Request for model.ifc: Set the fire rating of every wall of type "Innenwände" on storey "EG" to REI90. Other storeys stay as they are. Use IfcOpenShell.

First a look at what the model holds.

```python
import ifcopenshell
import ifcopenshell.util.element

model = ifcopenshell.open("model.ifc")
print(model.schema)
storey = next(s for s in model.by_type("IfcBuildingStorey") if s.Name == "EG")
walls = [e for e in ifcopenshell.util.element.get_decomposition(storey) if e.is_a("IfcWall")]
seen = {}
for e in walls:
    element_type = ifcopenshell.util.element.get_type(e)
    key = (element_type.Name if element_type != e and element_type else None, ifcopenshell.util.element.get_pset(e, "Pset_WallCommon", "FireRating"))
    seen[key] = seen.get(key, 0) + 1
for (name, value), count in sorted(seen.items(), key=str):
    print(count, "x", name, "|", value)
```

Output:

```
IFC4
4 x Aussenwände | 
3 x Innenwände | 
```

```python
import ifcopenshell
import ifcopenshell.api.pset
import ifcopenshell.util.element

model = ifcopenshell.open("model.ifc")

storey = next(s for s in model.by_type("IfcBuildingStorey") if s.Name == "EG")
walls = [e for e in ifcopenshell.util.element.get_decomposition(storey) if e.is_a("IfcWall")]

count = 0
for e in walls:
    element_type = ifcopenshell.util.element.get_type(e)
    if element_type in (None, e) or element_type.Name != "Innenwände":
        continue
    # add_pset returns the element's existing set when there is one.
    pset = ifcopenshell.api.pset.add_pset(model, product=e, name="Pset_WallCommon")
    ifcopenshell.api.pset.edit_pset(model, pset=pset, properties={"FireRating": "REI90"})
    count += 1

print(count, "walls updated")

model.write("model_rev.ifc")
```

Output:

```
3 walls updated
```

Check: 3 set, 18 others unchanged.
